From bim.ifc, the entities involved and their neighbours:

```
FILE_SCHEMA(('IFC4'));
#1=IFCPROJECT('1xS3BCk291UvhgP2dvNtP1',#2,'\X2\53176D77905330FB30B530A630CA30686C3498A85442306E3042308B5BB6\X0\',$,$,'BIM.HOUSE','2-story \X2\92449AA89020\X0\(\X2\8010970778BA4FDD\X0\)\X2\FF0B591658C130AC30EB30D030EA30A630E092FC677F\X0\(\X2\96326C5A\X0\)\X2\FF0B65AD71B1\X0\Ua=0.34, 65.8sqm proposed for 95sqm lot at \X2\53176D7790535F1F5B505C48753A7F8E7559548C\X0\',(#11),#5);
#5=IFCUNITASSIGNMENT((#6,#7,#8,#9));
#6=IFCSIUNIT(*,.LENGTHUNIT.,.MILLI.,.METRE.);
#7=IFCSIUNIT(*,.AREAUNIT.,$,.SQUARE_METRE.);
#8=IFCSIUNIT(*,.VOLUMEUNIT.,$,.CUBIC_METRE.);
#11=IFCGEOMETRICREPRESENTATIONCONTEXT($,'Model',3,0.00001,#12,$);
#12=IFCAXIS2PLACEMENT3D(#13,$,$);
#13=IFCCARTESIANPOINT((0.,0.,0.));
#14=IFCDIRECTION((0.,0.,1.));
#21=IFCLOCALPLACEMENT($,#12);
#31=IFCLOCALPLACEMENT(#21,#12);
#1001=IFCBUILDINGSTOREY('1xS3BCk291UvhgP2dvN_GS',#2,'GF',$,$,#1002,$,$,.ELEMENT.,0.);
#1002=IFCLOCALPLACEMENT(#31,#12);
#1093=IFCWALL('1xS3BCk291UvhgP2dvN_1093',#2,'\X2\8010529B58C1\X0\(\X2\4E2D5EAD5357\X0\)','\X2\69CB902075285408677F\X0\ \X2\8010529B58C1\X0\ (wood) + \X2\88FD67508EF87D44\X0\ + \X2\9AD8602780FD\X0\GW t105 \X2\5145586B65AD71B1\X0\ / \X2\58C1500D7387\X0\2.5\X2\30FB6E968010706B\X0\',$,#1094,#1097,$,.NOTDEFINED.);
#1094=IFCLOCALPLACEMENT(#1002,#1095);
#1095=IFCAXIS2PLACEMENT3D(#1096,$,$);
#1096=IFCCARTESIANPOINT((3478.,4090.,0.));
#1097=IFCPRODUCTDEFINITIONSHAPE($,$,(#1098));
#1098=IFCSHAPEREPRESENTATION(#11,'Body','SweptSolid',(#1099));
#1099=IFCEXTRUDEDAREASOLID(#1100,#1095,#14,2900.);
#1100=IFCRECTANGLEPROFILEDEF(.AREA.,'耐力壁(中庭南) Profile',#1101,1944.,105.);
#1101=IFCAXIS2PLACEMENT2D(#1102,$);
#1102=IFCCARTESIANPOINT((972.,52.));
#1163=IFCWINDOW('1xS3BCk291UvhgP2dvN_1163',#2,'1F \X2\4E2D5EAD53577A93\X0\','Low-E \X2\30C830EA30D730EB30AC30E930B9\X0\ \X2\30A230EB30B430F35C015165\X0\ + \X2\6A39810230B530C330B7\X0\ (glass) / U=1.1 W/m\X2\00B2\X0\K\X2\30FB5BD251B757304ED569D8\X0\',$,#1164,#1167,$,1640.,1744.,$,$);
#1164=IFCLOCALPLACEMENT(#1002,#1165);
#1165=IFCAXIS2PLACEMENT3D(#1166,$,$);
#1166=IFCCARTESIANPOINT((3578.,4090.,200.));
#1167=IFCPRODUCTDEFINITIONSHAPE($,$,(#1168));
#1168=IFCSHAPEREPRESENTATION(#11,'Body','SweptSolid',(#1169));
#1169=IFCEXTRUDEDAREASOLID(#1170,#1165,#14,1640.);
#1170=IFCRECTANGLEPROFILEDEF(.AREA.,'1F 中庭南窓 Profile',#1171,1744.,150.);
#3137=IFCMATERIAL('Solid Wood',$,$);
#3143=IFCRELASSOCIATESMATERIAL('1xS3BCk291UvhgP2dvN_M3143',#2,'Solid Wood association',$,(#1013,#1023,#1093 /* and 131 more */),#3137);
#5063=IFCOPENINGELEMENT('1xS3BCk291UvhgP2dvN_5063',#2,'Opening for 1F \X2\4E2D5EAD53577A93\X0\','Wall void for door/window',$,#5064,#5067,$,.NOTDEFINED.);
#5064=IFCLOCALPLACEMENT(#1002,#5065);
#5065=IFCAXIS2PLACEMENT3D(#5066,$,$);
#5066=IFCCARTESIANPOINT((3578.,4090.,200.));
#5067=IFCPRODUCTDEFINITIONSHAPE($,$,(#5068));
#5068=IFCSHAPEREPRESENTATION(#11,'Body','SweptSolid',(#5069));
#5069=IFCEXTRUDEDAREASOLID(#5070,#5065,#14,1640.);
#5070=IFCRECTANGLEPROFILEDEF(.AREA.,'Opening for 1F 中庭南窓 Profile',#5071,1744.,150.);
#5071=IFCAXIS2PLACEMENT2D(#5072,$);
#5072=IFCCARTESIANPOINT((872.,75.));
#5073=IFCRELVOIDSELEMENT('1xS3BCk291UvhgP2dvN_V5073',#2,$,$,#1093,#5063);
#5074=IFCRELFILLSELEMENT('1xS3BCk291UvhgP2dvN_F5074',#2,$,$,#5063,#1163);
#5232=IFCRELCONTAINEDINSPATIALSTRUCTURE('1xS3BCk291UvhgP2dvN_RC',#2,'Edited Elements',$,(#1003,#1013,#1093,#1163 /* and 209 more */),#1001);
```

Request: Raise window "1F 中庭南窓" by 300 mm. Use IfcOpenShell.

```python
import numpy as np
import ifcopenshell
import ifcopenshell.api.geometry
import ifcopenshell.util.placement
import ifcopenshell.util.unit

model = ifcopenshell.open("bim.ifc")
unit_scale = ifcopenshell.util.unit.calculate_unit_scale(model)

window = model.by_id(1163)
opening = window.FillsVoids[0].RelatingOpeningElement
dz = 0.3 / unit_scale

shift = np.array([0.0, 0.0, dz])
# The window is not placed relative to its opening, so move both.
for product in (opening, window):
    matrix = ifcopenshell.util.placement.get_local_placement(product.ObjectPlacement)
    matrix[:3, 3] += shift
    ifcopenshell.api.geometry.edit_object_placement(model, product=product, matrix=matrix, is_si=False)

print(f"moved by {dz * unit_scale:+.3f} m")

model.write("bim_edited.ifc")
```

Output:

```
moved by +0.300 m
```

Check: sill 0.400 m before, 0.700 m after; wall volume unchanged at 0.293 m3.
